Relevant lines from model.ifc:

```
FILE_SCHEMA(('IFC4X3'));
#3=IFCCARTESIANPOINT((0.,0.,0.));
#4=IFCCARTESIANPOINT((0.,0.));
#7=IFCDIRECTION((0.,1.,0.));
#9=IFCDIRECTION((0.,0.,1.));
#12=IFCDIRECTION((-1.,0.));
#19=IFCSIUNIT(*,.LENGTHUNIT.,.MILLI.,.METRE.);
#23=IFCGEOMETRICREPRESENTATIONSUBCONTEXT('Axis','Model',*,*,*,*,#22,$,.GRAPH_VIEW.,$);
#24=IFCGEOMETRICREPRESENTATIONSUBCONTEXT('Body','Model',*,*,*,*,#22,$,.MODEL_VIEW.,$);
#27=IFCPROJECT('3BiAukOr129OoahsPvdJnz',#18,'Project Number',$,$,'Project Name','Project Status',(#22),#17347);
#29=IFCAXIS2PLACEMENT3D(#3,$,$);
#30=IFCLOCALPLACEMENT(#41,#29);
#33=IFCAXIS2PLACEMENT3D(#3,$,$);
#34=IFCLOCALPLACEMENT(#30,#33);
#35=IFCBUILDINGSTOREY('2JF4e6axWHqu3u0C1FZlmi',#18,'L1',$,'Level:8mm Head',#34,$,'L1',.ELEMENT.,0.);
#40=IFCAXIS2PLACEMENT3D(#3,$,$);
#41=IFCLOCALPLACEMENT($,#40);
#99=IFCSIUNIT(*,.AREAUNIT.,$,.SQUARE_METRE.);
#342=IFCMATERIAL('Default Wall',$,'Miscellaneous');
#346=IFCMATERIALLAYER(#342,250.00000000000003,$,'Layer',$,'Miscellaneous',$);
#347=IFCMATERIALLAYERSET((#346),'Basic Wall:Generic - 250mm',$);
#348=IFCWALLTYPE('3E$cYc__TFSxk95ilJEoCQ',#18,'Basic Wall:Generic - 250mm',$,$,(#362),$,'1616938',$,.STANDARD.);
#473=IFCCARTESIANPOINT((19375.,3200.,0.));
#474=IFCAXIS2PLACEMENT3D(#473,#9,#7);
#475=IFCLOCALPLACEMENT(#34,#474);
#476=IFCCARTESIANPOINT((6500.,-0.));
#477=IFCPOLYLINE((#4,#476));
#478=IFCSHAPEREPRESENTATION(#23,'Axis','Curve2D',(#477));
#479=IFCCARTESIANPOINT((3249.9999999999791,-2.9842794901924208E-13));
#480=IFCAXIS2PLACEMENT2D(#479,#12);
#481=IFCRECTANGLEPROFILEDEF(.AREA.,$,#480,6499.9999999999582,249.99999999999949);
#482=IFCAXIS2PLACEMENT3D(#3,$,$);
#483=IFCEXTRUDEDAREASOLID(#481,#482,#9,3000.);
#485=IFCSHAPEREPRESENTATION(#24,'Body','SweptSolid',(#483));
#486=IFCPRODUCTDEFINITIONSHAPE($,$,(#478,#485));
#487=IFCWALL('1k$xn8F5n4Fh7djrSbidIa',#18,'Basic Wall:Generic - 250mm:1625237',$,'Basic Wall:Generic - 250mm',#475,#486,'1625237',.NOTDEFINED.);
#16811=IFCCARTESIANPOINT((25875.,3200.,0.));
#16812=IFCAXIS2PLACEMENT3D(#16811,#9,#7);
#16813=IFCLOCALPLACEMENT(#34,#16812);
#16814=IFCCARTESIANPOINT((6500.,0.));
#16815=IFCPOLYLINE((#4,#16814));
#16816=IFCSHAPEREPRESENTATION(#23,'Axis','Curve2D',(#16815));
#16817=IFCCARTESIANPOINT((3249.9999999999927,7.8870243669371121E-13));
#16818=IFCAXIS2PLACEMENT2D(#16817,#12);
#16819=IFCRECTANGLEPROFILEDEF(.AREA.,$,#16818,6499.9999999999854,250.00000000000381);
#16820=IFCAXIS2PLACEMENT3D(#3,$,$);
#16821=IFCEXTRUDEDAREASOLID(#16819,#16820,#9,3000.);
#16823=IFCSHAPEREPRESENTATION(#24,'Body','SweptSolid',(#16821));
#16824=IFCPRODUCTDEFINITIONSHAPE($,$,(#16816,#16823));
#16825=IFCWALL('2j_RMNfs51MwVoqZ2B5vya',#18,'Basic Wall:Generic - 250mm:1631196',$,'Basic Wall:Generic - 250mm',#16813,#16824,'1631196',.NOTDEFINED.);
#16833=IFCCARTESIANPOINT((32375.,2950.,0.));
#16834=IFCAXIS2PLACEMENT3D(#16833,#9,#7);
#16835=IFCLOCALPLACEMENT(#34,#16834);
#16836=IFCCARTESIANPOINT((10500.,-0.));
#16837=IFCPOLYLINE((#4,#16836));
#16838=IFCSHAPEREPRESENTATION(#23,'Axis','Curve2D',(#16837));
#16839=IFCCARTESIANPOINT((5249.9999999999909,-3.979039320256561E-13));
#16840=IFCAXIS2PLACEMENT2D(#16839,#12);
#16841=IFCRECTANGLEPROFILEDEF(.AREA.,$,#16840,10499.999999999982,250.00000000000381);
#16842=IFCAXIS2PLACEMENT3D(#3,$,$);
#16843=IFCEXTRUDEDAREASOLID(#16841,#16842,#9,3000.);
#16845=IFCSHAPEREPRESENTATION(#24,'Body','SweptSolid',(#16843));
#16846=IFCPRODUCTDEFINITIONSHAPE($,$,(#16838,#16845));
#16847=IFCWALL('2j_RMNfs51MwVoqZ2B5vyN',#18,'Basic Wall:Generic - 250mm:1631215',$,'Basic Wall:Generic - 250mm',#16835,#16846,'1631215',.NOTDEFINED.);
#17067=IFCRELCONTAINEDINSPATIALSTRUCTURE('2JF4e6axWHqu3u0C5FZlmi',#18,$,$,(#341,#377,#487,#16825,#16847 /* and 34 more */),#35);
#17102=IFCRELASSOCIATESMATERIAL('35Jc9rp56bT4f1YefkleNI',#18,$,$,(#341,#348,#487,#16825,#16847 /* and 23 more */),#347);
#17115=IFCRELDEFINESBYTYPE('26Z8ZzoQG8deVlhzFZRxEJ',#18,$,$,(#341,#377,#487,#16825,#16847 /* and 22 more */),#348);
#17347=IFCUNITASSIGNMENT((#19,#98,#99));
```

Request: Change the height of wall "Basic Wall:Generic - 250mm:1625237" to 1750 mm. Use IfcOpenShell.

```python
import ifcopenshell
import ifcopenshell.geom
import ifcopenshell.util.representation
import ifcopenshell.util.shape
import ifcopenshell.util.unit

model = ifcopenshell.open("model.ifc")
unit_scale = ifcopenshell.util.unit.calculate_unit_scale(model)
settings = ifcopenshell.geom.settings()


def volume(element):
    """Net volume in cubic metres, openings subtracted."""
    shape = ifcopenshell.geom.create_shape(settings, element)
    return ifcopenshell.util.shape.get_volume(shape.geometry)


wall = model.by_guid("1k$xn8F5n4Fh7djrSbidIa")
before = volume(wall)

body = ifcopenshell.util.representation.get_representation(wall, "Model", "Body")
solid = body.Items[0]
old_height = solid.Depth
solid.Depth = 1.75 / unit_scale
after = volume(wall)

print(f"height {old_height:g} -> {solid.Depth:g}, volume {before:.3f} -> {after:.3f} m3")

model.write("model-out.ifc")
```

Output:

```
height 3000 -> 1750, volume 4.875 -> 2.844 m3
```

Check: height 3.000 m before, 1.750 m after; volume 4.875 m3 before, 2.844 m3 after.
